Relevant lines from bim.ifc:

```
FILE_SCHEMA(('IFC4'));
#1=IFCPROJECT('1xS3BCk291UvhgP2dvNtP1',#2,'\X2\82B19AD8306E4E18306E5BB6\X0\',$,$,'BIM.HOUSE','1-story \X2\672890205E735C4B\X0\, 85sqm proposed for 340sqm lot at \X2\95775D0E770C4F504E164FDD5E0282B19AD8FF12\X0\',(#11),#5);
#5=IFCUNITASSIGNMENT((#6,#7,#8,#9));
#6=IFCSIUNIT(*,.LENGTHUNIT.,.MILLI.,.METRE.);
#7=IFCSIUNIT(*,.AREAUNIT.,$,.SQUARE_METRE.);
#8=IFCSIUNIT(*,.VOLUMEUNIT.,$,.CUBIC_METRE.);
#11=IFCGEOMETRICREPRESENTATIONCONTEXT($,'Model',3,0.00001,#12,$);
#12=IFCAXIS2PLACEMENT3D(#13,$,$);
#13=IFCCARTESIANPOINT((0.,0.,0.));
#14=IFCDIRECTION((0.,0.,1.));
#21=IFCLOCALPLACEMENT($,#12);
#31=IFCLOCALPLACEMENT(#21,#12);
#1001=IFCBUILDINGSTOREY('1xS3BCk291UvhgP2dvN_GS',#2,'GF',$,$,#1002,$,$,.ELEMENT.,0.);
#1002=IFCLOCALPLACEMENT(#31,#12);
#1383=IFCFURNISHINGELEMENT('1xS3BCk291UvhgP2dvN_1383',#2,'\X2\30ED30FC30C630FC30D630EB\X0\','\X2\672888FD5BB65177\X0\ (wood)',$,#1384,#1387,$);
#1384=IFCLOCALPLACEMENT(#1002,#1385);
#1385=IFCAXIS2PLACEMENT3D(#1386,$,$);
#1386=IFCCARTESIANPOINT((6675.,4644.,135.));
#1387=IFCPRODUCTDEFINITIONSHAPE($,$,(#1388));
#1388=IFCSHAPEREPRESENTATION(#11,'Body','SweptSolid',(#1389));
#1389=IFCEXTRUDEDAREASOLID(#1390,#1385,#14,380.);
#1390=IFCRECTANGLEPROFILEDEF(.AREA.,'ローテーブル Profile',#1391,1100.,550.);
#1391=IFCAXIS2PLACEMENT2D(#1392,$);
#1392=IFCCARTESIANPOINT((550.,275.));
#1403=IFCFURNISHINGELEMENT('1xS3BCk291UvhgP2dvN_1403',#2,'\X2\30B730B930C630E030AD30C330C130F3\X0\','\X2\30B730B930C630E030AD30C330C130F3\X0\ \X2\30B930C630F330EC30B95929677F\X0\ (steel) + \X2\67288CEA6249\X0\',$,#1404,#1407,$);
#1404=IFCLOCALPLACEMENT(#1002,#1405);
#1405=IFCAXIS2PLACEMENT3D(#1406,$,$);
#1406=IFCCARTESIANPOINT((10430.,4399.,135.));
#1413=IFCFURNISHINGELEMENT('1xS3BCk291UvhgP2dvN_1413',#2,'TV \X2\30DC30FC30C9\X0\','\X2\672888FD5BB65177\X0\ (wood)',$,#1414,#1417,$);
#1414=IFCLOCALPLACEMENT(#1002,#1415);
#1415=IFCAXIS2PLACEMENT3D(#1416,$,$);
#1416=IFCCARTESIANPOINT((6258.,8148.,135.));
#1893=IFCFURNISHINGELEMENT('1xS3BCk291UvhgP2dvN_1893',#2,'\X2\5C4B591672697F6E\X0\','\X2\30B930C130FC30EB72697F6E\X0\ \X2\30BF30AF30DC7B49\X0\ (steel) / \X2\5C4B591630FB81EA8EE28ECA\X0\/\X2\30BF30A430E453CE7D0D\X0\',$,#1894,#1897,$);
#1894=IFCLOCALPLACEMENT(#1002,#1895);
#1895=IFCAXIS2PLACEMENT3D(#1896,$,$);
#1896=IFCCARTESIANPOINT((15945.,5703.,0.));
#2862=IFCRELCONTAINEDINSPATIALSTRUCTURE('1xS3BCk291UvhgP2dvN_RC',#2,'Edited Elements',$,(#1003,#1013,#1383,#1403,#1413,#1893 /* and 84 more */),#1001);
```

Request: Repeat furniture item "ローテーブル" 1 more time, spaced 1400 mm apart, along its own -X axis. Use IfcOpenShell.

```python
import ifcopenshell
import ifcopenshell.api.geometry
import ifcopenshell.api.root
import ifcopenshell.util.element
import ifcopenshell.util.placement
import ifcopenshell.util.unit

model = ifcopenshell.open("bim.ifc")
unit_scale = ifcopenshell.util.unit.calculate_unit_scale(model)


def reuse_history(source, copy):
    """copy_class also copies each property set's owner history, people and application; keep the originals."""
    for rel in copy.IsDefinedBy:
        if rel.is_a("IfcRelDefinesByProperties") and (history := rel.RelatingPropertyDefinition.OwnerHistory):
            rel.RelatingPropertyDefinition.OwnerHistory = source.OwnerHistory
            ifcopenshell.util.element.remove_deep2(model, history)


source = model.by_guid("1xS3BCk291UvhgP2dvN_1383")
base = ifcopenshell.util.placement.get_local_placement(source.ObjectPlacement)
step = -base[:3, 0] * 1.4 / unit_scale

for i in range(1, 2):
    copy = ifcopenshell.api.root.copy_class(model, product=source)
    copy.Representation = ifcopenshell.util.element.copy_deep(
        model, source.Representation, exclude=["IfcGeometricRepresentationContext", "IfcRepresentationMap"]
    )
    reuse_history(source, copy)
    matrix = base.copy()
    matrix[:3, 3] += i * step
    print("added at", matrix[:3, 3].round(3) + 0.0)
    ifcopenshell.api.geometry.edit_object_placement(model, product=copy, matrix=matrix, is_si=False)

model.write("bim_v2.ifc")
```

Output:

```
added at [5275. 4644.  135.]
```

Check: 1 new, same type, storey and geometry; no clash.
